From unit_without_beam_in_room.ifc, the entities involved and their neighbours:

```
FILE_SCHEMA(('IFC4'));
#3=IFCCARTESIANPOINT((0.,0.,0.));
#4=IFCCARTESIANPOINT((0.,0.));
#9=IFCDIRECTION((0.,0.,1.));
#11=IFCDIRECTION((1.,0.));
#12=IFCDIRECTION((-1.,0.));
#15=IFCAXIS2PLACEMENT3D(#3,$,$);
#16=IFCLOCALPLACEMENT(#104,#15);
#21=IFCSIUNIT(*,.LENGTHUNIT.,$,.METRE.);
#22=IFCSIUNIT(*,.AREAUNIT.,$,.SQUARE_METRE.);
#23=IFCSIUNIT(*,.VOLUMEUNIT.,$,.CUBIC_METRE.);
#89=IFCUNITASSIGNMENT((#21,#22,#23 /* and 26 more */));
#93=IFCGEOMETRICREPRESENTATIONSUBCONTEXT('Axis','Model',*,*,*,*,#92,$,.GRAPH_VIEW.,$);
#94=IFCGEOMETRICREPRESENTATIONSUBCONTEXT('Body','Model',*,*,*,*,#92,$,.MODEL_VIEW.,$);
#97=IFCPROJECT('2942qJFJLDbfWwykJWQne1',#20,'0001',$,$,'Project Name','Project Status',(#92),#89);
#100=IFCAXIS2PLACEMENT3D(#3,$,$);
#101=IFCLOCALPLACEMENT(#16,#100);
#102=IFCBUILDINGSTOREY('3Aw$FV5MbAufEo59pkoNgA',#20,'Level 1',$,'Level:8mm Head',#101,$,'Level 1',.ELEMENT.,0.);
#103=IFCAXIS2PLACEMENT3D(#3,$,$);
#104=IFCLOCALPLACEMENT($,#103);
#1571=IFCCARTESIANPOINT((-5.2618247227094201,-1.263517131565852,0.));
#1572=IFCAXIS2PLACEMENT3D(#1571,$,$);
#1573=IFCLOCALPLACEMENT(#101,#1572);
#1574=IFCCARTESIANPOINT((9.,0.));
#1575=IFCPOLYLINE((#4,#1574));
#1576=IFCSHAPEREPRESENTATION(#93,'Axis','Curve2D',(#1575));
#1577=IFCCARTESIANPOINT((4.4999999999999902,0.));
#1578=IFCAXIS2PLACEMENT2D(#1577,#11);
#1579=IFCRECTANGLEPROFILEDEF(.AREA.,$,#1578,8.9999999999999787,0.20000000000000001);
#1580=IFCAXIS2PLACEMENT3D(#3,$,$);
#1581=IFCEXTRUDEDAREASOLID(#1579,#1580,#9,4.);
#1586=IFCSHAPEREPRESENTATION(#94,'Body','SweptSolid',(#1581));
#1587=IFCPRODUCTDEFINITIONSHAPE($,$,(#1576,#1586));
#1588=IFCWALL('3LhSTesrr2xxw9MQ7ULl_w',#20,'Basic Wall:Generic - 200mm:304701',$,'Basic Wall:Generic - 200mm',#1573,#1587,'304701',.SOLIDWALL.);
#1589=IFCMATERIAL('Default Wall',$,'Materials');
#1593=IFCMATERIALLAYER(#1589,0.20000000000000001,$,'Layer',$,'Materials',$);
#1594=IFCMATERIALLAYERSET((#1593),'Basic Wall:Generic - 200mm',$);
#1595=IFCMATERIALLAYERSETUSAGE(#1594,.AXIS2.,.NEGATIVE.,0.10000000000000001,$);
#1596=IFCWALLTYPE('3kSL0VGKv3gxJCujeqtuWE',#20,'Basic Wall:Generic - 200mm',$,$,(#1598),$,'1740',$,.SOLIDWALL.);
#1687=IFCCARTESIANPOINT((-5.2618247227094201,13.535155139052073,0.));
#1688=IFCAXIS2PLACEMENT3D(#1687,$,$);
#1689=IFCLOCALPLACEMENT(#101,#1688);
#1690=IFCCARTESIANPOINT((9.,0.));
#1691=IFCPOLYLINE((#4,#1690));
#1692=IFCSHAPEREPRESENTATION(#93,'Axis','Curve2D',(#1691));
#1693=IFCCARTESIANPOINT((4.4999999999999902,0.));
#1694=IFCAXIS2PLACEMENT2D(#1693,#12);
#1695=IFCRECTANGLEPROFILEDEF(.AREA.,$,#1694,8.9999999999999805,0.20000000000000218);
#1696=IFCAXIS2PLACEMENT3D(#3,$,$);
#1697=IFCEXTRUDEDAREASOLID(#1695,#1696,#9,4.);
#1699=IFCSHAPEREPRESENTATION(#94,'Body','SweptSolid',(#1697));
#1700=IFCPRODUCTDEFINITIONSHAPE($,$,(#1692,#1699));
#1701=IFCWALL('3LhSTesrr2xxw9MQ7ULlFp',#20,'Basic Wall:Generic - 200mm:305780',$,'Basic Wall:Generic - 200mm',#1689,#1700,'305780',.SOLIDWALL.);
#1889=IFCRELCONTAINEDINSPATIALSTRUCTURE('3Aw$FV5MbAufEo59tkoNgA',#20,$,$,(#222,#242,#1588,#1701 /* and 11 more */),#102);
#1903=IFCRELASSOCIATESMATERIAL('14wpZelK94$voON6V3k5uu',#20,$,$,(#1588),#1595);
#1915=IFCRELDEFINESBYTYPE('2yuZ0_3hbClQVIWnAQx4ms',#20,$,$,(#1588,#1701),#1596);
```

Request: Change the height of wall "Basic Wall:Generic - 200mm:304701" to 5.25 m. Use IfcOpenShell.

```python
import ifcopenshell
import ifcopenshell.geom
import ifcopenshell.util.representation
import ifcopenshell.util.shape
import ifcopenshell.util.unit

model = ifcopenshell.open("unit_without_beam_in_room.ifc")
unit_scale = ifcopenshell.util.unit.calculate_unit_scale(model)
settings = ifcopenshell.geom.settings()


def volume(element):
    """Net volume in cubic metres, openings subtracted."""
    shape = ifcopenshell.geom.create_shape(settings, element)
    return ifcopenshell.util.shape.get_volume(shape.geometry)


wall = model.by_guid("3LhSTesrr2xxw9MQ7ULl_w")
before = volume(wall)

body = ifcopenshell.util.representation.get_representation(wall, "Model", "Body")
solid = body.Items[0]
old_height = solid.Depth
solid.Depth = 5.25 / unit_scale
after = volume(wall)

print(f"height {old_height:g} -> {solid.Depth:g}, volume {before:.3f} -> {after:.3f} m3")

model.write("unit_without_beam_in_room-out.ifc")
```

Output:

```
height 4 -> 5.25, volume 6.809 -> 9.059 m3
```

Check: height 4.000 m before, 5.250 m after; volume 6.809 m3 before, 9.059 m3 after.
